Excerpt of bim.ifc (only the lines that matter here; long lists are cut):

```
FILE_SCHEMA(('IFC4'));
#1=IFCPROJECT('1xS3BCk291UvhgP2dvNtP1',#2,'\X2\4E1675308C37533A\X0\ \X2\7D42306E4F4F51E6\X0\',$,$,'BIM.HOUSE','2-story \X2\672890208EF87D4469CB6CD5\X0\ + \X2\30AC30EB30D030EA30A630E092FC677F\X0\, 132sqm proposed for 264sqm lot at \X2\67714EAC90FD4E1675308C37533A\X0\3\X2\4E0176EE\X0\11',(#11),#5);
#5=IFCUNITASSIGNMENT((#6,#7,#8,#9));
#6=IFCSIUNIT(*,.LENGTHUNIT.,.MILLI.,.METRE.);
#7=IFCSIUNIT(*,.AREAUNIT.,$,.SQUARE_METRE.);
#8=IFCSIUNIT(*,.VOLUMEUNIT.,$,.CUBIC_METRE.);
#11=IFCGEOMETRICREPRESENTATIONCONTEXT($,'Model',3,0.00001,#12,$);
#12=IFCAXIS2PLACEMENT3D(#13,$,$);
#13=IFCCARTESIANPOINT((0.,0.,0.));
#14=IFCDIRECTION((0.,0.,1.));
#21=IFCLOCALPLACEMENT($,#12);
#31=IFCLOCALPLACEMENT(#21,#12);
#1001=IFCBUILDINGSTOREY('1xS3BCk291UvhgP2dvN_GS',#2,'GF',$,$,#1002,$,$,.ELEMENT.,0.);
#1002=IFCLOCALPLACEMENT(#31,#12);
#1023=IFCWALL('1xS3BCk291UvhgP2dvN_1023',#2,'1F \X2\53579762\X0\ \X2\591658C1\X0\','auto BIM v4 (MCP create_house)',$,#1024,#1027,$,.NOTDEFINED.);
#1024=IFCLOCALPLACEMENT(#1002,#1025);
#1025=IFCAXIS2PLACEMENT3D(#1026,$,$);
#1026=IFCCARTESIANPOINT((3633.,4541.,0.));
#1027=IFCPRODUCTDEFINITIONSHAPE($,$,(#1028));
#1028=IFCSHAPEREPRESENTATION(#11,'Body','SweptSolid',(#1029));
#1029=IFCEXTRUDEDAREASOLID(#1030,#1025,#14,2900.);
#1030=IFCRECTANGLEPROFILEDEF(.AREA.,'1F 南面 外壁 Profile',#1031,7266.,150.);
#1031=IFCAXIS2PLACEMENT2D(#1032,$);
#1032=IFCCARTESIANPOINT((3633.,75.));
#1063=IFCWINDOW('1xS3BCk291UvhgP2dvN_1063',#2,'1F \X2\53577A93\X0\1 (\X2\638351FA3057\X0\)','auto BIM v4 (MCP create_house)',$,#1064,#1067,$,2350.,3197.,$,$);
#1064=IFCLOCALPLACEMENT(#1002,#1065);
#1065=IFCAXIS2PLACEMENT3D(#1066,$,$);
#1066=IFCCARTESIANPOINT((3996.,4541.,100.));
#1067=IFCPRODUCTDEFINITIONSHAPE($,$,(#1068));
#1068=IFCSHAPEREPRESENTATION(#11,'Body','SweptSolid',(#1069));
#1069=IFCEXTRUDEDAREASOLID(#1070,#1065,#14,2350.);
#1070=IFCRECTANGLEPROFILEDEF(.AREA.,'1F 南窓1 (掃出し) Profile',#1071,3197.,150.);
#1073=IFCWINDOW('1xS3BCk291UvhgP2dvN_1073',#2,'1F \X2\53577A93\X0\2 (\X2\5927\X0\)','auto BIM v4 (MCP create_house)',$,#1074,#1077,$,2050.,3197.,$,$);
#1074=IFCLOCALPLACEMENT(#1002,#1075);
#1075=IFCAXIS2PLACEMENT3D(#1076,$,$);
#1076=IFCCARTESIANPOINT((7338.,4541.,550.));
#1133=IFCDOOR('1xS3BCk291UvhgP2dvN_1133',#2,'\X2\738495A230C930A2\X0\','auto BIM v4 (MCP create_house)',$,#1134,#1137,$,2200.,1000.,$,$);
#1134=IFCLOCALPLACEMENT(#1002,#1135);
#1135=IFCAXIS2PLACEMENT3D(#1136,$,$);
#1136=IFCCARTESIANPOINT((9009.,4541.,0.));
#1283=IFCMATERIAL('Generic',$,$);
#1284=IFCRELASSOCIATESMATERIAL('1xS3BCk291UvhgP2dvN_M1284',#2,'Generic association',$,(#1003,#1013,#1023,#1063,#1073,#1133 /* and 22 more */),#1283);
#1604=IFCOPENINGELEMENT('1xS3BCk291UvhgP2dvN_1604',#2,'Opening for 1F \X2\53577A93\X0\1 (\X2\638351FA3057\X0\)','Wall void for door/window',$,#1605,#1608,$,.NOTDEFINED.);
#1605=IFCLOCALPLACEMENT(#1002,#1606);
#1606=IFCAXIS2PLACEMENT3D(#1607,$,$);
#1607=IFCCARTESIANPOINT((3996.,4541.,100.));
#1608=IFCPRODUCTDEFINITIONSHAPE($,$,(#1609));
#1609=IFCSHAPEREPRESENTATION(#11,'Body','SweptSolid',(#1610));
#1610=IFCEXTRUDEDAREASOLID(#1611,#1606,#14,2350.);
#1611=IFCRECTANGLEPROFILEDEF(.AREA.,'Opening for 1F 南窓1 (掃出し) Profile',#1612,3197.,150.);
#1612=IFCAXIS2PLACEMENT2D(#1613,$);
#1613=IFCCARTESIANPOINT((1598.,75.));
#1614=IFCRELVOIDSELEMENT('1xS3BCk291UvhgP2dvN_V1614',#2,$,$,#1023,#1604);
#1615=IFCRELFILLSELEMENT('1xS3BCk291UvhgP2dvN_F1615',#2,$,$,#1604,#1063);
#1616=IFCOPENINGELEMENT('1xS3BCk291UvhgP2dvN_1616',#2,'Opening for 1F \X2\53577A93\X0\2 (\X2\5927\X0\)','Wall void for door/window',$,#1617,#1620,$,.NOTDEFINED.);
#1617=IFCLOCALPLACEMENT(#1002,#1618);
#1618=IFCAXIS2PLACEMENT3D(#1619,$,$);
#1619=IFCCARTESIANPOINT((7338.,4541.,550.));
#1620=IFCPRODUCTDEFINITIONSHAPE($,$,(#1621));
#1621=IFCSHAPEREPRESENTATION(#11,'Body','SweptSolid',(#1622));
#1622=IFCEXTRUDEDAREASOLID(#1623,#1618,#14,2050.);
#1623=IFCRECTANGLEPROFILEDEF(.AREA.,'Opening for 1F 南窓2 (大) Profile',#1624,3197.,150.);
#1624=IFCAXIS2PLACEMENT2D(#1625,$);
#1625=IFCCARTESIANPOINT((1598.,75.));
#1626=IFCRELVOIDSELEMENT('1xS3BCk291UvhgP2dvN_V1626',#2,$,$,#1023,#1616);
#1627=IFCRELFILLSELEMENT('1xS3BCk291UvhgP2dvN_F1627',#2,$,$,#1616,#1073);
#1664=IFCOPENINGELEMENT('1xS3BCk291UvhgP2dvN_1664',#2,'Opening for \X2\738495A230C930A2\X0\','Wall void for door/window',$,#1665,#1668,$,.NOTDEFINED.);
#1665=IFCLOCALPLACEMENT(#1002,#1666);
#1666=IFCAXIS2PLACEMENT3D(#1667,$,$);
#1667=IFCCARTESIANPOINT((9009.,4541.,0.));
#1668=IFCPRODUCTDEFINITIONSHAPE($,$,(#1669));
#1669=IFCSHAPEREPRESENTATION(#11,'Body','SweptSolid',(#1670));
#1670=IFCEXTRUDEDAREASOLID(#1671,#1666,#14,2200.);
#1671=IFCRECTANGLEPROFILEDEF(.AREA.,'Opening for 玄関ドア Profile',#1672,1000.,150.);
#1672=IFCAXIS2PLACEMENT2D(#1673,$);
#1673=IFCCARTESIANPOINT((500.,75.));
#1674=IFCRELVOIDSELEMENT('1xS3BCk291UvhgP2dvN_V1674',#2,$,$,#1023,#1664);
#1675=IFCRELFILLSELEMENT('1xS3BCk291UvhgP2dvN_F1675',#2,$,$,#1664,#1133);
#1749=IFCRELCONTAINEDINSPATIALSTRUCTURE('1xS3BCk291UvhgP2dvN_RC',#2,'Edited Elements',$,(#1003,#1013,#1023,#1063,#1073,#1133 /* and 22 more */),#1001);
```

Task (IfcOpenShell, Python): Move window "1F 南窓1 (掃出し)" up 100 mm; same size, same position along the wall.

```python
import numpy as np
import ifcopenshell
import ifcopenshell.api.geometry
import ifcopenshell.util.placement
import ifcopenshell.util.unit

model = ifcopenshell.open("bim.ifc")
unit_scale = ifcopenshell.util.unit.calculate_unit_scale(model)

window = model.by_guid("1xS3BCk291UvhgP2dvN_1063")
opening = window.FillsVoids[0].RelatingOpeningElement
dz = 0.1 / unit_scale

shift = np.array([0.0, 0.0, dz])
# The window is not placed relative to its opening, so move both.
for product in (opening, window):
    matrix = ifcopenshell.util.placement.get_local_placement(product.ObjectPlacement)
    matrix[:3, 3] += shift
    ifcopenshell.api.geometry.edit_object_placement(model, product=product, matrix=matrix, is_si=False)

print(f"moved by {dz * unit_scale:+.3f} m")

model.write("bim_v2.ifc")
```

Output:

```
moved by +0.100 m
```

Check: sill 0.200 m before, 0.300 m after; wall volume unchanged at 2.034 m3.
